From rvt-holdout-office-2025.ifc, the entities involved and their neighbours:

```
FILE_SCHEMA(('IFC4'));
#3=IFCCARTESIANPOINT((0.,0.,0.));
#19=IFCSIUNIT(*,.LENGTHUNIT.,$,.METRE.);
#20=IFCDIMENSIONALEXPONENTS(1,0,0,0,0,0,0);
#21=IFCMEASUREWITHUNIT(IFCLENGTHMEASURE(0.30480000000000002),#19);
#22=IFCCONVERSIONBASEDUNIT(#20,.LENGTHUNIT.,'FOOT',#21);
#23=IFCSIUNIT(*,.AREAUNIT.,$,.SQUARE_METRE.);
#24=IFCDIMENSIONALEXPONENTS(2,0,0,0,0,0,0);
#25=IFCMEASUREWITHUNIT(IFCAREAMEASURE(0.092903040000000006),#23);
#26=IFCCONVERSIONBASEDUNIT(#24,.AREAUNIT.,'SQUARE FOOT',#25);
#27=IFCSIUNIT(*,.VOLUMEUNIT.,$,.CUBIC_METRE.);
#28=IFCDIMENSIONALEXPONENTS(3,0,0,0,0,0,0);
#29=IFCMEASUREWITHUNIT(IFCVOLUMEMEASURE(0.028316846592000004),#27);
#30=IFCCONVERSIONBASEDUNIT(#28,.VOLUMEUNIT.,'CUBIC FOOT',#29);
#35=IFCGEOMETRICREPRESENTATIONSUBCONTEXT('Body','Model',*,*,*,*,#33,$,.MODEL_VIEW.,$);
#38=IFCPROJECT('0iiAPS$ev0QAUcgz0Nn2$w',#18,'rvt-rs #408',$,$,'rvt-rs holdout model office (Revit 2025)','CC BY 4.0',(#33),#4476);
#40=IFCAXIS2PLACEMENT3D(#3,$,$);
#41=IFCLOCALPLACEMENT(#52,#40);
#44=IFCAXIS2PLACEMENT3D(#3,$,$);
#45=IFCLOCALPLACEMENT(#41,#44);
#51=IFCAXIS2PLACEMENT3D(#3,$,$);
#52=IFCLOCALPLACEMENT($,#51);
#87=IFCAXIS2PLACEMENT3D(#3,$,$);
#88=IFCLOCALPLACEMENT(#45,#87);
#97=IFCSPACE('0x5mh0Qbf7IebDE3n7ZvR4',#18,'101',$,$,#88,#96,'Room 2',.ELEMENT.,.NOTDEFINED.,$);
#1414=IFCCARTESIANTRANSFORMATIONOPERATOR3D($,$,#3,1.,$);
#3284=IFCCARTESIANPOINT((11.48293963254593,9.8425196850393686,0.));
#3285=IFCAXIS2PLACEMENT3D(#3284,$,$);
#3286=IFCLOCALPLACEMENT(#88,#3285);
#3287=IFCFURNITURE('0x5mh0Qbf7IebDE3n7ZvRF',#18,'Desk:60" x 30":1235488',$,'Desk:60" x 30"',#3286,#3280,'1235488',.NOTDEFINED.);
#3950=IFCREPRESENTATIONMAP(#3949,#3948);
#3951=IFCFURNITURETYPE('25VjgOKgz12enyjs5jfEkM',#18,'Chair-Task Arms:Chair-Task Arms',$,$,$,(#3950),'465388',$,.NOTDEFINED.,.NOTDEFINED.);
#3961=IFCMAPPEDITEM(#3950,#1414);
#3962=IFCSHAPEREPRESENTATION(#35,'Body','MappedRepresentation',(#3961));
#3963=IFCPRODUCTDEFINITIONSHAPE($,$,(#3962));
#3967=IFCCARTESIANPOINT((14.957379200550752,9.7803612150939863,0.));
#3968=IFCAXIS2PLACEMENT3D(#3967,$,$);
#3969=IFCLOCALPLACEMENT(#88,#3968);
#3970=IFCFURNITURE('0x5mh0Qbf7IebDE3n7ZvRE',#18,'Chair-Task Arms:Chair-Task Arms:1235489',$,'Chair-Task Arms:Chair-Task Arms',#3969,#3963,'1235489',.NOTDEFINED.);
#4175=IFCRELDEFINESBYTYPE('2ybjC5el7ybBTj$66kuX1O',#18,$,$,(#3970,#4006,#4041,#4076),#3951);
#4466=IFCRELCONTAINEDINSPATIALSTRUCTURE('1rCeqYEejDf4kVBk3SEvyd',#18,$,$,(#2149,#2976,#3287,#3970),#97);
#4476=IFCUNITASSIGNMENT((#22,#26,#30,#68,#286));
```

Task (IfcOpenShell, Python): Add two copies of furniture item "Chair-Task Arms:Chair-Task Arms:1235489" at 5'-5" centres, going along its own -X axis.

```python
import ifcopenshell
import ifcopenshell.api.geometry
import ifcopenshell.api.root
import ifcopenshell.util.element
import ifcopenshell.util.placement
import ifcopenshell.util.unit

model = ifcopenshell.open("rvt-holdout-office-2025.ifc")
unit_scale = ifcopenshell.util.unit.calculate_unit_scale(model)


def reuse_history(source, copy):
    """copy_class also copies each property set's owner history, people and application; keep the originals."""
    for rel in copy.IsDefinedBy:
        if rel.is_a("IfcRelDefinesByProperties") and (history := rel.RelatingPropertyDefinition.OwnerHistory):
            rel.RelatingPropertyDefinition.OwnerHistory = source.OwnerHistory
            ifcopenshell.util.element.remove_deep2(model, history)


source = model.by_guid("0x5mh0Qbf7IebDE3n7ZvRE")
base = ifcopenshell.util.placement.get_local_placement(source.ObjectPlacement)
step = -base[:3, 0] * 65 * 0.0254 / unit_scale

for i in range(1, 3):
    copy = ifcopenshell.api.root.copy_class(model, product=source)
    copy.Representation = ifcopenshell.util.element.copy_deep(
        model, source.Representation, exclude=["IfcGeometricRepresentationContext", "IfcRepresentationMap"]
    )
    copy.Name = "Chair-Task Arms:Chair-Task Arms"
    copy.Tag = None
    reuse_history(source, copy)
    matrix = base.copy()
    matrix[:3, 3] += i * step
    print("added at", matrix[:3, 3].round(3) + 0.0)
    ifcopenshell.api.geometry.edit_object_placement(model, product=copy, matrix=matrix, is_si=False)

model.write("rvt-holdout-office-2025_edited.ifc")
```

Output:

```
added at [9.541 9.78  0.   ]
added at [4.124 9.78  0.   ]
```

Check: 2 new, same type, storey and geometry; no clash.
